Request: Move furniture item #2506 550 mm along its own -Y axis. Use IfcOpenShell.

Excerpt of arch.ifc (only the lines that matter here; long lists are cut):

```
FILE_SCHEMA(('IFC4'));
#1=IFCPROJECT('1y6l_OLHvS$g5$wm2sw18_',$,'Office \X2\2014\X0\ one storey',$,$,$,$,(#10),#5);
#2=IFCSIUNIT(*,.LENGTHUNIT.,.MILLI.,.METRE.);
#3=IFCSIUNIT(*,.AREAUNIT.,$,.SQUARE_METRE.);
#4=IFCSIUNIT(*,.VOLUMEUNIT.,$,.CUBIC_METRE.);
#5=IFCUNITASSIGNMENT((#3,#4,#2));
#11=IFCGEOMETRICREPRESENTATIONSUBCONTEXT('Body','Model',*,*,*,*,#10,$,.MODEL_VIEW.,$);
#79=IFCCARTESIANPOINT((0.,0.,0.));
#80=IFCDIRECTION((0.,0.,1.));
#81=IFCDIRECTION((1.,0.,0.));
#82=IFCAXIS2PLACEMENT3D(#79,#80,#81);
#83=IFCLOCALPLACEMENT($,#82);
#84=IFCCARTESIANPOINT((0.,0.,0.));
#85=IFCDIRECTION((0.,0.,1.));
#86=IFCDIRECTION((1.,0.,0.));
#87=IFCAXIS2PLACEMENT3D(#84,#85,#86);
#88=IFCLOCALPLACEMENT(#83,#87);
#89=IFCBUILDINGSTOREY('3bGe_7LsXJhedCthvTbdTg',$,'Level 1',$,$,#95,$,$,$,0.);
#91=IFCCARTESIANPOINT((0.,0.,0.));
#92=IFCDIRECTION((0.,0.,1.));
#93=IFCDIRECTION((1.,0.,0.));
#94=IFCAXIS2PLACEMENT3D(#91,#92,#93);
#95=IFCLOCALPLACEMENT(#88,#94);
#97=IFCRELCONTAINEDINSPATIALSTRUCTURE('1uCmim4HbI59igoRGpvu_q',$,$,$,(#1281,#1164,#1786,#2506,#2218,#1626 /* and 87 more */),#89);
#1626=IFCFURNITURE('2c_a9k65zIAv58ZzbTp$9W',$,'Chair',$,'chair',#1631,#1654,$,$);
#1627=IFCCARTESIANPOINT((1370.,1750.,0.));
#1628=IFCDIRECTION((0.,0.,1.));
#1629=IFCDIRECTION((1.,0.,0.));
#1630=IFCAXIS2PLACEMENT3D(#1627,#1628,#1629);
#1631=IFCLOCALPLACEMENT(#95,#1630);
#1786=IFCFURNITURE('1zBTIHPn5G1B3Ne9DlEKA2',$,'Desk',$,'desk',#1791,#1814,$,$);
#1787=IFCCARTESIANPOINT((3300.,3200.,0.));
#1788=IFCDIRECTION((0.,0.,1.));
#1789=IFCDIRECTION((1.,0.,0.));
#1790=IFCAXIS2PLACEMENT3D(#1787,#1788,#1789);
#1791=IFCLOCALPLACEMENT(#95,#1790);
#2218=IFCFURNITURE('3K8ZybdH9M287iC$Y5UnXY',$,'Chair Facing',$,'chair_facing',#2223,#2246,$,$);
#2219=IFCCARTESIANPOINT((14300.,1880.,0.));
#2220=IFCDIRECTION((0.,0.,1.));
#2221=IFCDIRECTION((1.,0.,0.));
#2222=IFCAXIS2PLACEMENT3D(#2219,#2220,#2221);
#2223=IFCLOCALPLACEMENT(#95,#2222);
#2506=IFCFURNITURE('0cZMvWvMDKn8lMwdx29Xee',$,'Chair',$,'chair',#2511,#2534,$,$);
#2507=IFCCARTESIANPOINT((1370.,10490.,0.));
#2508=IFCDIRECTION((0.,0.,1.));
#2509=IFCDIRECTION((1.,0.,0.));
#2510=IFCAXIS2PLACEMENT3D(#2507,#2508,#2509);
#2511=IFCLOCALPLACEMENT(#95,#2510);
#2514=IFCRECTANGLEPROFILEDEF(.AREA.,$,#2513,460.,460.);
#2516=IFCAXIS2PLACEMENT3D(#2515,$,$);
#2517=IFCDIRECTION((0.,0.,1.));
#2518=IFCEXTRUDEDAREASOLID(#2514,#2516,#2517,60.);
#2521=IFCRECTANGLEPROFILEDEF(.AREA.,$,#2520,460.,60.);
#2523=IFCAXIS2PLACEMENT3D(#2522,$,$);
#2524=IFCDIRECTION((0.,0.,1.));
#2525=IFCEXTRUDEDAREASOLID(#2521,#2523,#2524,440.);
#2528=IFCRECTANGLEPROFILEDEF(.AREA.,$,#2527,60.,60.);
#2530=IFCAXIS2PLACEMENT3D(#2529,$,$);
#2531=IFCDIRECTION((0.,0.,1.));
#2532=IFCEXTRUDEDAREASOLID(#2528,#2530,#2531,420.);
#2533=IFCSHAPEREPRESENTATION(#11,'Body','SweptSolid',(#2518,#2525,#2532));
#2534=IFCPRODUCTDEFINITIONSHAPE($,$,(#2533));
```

```python
import ifcopenshell
import ifcopenshell.api.geometry
import ifcopenshell.util.placement
import ifcopenshell.util.unit

model = ifcopenshell.open("arch.ifc")
unit_scale = ifcopenshell.util.unit.calculate_unit_scale(model)

item = model.by_guid("0cZMvWvMDKn8lMwdx29Xee")
matrix = ifcopenshell.util.placement.get_local_placement(item.ObjectPlacement)
matrix[:3, 3] -= matrix[:3, 1] * 0.55 / unit_scale
ifcopenshell.api.geometry.edit_object_placement(model, product=item, matrix=matrix, is_si=False)

print(ifcopenshell.util.placement.get_local_placement(item.ObjectPlacement).round(3) + 0.0)

model.write("arch_updated.ifc")
```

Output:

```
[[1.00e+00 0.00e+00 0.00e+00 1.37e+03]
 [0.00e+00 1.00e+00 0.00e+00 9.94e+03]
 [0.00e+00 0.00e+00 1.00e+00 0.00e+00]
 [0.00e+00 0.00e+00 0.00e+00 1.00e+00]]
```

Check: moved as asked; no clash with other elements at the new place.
